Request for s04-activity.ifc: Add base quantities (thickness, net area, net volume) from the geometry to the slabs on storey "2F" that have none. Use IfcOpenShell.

First a look at what the model holds.

```python
import ifcopenshell
import ifcopenshell.util.element
import ifcopenshell.util.unit

model = ifcopenshell.open("s04-activity.ifc")
print(model.schema)
for unit_type in ("LENGTHUNIT", "AREAUNIT", "VOLUMEUNIT"):
    print(unit_type, ifcopenshell.util.unit.calculate_unit_scale(model, unit_type))
storey = next(s for s in model.by_type("IfcBuildingStorey") if s.Name == "2F")
slabs = [e for e in ifcopenshell.util.element.get_decomposition(storey) if e.is_a("IfcSlab")]
for e in sorted(slabs, key=lambda e: e.id()):
    print(e.id(), e.is_a(), e.Name, list(ifcopenshell.util.element.get_psets(e, qtos_only=True)), sep=" | ")
```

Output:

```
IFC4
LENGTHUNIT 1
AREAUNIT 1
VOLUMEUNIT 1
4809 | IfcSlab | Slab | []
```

```python
import ifcopenshell
import ifcopenshell.api.pset
import ifcopenshell.geom
import ifcopenshell.util.element
import ifcopenshell.util.shape
import ifcopenshell.util.unit

model = ifcopenshell.open("s04-activity.ifc")
unit_scale = ifcopenshell.util.unit.calculate_unit_scale(model)
area_scale = ifcopenshell.util.unit.calculate_unit_scale(model, "AREAUNIT")
volume_scale = ifcopenshell.util.unit.calculate_unit_scale(model, "VOLUMEUNIT")
settings = ifcopenshell.geom.settings()

storey = next(s for s in model.by_type("IfcBuildingStorey") if s.Name == "2F")
slabs = [e for e in ifcopenshell.util.element.get_decomposition(storey) if e.is_a("IfcSlab")]

for e in sorted(slabs, key=lambda e: e.id()):
    if ifcopenshell.util.element.get_psets(e, qtos_only=True, should_inherit=False):
        continue
    # Geometry comes back in metres, in the element's own axes.
    shape = ifcopenshell.geom.create_shape(settings, e)
    values = {
        "Width": ifcopenshell.util.shape.get_z(shape.geometry) / unit_scale,
        "NetArea": ifcopenshell.util.shape.get_footprint_area(shape.geometry) / area_scale,
        "NetVolume": ifcopenshell.util.shape.get_volume(shape.geometry) / volume_scale,
    }
    qto = ifcopenshell.api.pset.add_qto(model, product=e, name="Qto_SlabBaseQuantities")
    ifcopenshell.api.pset.edit_qto(model, qto=qto, properties=values)
    print(e.id(), {k: round(v, 3) for k, v in values.items()})

model.write("s04-activity_v2.ifc")
```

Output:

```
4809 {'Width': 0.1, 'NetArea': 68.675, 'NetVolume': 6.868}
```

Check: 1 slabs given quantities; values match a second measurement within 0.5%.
